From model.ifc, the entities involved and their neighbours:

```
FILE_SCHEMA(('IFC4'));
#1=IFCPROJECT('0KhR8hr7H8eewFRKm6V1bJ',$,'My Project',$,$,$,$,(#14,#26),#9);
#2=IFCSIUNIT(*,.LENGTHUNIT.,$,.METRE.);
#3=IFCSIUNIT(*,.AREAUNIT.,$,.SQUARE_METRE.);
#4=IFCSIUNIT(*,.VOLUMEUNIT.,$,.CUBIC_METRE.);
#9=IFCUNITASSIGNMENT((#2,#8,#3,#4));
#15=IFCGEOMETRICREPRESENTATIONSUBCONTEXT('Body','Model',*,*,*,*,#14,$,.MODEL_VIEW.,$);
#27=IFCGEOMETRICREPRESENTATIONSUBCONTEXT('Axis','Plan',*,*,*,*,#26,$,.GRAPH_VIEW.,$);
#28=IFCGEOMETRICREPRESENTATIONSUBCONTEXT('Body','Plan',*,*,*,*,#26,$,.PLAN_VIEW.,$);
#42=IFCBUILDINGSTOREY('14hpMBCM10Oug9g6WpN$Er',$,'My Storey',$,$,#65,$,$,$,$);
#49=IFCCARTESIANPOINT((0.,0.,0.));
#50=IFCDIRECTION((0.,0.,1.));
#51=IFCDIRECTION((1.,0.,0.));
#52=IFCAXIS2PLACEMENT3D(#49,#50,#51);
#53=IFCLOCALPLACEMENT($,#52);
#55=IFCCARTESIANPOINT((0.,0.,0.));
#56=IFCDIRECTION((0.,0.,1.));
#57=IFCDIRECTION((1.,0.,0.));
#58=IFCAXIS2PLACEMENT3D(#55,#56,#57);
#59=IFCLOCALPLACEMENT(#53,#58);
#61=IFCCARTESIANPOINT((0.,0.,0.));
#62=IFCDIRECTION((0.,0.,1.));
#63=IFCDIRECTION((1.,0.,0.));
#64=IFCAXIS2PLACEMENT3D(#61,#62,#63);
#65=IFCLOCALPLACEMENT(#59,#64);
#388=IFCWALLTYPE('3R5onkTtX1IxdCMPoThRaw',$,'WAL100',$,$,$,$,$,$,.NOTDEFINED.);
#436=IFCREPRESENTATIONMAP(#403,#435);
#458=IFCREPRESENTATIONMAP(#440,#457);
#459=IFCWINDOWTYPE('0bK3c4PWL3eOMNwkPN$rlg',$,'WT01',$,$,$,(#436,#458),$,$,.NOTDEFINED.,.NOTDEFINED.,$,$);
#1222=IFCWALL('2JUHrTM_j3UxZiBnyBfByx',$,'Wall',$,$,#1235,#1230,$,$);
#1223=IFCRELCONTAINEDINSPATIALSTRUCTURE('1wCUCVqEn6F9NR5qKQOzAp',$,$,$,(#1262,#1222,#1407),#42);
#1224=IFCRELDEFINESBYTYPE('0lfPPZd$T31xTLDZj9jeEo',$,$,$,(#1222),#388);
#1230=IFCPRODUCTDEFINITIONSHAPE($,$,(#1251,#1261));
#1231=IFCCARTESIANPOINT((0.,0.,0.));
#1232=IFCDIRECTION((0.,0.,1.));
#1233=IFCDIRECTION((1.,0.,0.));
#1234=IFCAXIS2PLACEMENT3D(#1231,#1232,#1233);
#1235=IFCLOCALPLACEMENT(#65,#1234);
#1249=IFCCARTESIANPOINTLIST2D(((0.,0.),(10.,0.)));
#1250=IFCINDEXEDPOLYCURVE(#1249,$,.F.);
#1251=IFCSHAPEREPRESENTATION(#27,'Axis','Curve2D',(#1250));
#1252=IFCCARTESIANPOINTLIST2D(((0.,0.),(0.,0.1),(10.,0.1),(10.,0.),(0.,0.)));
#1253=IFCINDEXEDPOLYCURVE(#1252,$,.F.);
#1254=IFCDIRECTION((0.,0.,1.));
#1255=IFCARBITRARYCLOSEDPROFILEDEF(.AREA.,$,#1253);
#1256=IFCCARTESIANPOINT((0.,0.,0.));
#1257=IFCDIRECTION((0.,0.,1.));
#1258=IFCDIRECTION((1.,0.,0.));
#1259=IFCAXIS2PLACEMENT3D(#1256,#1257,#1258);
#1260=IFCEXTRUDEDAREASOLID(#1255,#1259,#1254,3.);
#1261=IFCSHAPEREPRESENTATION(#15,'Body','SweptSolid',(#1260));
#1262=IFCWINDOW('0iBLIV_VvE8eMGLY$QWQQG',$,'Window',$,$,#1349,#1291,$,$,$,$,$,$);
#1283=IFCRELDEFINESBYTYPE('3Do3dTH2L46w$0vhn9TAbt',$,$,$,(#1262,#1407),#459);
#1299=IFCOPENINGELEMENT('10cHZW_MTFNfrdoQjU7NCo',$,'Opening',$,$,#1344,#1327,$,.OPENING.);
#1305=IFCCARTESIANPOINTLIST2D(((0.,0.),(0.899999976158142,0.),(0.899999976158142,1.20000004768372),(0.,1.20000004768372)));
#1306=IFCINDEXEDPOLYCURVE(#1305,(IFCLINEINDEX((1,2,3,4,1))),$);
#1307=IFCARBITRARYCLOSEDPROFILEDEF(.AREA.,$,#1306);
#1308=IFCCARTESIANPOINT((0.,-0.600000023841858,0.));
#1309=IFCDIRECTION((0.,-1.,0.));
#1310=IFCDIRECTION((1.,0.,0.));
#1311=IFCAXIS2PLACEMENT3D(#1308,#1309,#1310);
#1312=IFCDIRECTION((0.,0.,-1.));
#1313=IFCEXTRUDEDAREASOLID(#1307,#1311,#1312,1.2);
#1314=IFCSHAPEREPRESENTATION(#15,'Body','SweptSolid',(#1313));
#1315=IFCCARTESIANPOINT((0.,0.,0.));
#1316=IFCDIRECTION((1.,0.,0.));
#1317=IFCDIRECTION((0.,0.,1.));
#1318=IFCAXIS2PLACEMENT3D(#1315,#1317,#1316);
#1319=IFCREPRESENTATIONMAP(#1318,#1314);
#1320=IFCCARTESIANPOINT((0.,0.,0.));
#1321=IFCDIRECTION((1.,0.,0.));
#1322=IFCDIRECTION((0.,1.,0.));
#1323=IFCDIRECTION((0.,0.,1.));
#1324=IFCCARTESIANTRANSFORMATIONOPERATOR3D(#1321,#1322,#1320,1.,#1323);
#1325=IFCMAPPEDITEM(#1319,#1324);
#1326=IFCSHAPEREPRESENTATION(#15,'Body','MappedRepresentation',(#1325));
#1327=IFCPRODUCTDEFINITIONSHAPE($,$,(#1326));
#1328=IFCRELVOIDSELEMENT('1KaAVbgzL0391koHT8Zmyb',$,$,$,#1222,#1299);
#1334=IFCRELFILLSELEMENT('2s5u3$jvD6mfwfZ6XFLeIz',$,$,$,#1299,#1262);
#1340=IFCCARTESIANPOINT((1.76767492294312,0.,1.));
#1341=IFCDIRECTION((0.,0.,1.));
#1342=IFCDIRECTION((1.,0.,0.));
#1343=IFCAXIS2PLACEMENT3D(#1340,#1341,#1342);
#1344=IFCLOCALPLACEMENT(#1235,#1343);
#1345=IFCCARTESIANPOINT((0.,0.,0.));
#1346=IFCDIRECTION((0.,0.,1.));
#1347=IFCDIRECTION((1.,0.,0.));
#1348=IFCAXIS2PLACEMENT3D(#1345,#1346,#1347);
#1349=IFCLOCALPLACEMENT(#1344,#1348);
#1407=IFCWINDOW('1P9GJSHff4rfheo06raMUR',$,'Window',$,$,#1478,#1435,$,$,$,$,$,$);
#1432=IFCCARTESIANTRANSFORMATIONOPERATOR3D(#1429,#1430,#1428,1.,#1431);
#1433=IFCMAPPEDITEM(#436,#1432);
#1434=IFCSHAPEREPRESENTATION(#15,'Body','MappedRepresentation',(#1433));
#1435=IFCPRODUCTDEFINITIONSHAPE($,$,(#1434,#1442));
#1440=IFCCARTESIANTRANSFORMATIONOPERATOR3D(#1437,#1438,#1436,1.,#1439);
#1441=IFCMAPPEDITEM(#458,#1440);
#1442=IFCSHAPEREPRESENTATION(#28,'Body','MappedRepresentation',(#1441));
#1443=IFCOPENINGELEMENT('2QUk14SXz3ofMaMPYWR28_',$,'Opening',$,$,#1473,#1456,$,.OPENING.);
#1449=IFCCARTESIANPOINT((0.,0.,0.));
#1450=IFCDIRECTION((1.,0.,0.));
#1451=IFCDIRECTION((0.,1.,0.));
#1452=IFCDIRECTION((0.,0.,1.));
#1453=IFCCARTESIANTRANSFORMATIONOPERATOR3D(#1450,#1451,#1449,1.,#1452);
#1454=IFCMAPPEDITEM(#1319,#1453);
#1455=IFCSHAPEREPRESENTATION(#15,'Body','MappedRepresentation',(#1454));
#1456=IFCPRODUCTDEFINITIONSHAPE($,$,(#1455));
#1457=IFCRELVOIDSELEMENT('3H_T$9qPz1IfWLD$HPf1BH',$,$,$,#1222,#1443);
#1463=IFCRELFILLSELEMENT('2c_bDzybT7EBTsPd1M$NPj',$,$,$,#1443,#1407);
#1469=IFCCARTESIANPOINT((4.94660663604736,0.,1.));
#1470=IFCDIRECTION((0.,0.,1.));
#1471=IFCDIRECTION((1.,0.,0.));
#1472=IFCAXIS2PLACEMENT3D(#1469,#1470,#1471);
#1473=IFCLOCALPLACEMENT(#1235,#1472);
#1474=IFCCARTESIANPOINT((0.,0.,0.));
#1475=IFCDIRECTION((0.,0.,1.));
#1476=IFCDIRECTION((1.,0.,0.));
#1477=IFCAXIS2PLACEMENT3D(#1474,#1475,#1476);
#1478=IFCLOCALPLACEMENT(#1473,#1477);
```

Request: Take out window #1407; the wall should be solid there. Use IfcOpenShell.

```python
import ifcopenshell
import ifcopenshell.api.feature
import ifcopenshell.api.root
import ifcopenshell.geom
import ifcopenshell.util.shape

model = ifcopenshell.open("model.ifc")
settings = ifcopenshell.geom.settings()


def volume(element):
    """Net volume in cubic metres, openings subtracted."""
    shape = ifcopenshell.geom.create_shape(settings, element)
    return ifcopenshell.util.shape.get_volume(shape.geometry)


window = model.by_guid("1P9GJSHff4rfheo06raMUR")
opening = window.FillsVoids[0].RelatingOpeningElement
wall = opening.VoidsElements[0].RelatingBuildingElement
before = volume(wall)

ifcopenshell.api.root.remove_product(model, product=window)
ifcopenshell.api.feature.remove_feature(model, feature=opening)

after = volume(wall)

print(f"wall volume {before:.3f} -> {after:.3f} m3")

model.write("model-out.ifc")
```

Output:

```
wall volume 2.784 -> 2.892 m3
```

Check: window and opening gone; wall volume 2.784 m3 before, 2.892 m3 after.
